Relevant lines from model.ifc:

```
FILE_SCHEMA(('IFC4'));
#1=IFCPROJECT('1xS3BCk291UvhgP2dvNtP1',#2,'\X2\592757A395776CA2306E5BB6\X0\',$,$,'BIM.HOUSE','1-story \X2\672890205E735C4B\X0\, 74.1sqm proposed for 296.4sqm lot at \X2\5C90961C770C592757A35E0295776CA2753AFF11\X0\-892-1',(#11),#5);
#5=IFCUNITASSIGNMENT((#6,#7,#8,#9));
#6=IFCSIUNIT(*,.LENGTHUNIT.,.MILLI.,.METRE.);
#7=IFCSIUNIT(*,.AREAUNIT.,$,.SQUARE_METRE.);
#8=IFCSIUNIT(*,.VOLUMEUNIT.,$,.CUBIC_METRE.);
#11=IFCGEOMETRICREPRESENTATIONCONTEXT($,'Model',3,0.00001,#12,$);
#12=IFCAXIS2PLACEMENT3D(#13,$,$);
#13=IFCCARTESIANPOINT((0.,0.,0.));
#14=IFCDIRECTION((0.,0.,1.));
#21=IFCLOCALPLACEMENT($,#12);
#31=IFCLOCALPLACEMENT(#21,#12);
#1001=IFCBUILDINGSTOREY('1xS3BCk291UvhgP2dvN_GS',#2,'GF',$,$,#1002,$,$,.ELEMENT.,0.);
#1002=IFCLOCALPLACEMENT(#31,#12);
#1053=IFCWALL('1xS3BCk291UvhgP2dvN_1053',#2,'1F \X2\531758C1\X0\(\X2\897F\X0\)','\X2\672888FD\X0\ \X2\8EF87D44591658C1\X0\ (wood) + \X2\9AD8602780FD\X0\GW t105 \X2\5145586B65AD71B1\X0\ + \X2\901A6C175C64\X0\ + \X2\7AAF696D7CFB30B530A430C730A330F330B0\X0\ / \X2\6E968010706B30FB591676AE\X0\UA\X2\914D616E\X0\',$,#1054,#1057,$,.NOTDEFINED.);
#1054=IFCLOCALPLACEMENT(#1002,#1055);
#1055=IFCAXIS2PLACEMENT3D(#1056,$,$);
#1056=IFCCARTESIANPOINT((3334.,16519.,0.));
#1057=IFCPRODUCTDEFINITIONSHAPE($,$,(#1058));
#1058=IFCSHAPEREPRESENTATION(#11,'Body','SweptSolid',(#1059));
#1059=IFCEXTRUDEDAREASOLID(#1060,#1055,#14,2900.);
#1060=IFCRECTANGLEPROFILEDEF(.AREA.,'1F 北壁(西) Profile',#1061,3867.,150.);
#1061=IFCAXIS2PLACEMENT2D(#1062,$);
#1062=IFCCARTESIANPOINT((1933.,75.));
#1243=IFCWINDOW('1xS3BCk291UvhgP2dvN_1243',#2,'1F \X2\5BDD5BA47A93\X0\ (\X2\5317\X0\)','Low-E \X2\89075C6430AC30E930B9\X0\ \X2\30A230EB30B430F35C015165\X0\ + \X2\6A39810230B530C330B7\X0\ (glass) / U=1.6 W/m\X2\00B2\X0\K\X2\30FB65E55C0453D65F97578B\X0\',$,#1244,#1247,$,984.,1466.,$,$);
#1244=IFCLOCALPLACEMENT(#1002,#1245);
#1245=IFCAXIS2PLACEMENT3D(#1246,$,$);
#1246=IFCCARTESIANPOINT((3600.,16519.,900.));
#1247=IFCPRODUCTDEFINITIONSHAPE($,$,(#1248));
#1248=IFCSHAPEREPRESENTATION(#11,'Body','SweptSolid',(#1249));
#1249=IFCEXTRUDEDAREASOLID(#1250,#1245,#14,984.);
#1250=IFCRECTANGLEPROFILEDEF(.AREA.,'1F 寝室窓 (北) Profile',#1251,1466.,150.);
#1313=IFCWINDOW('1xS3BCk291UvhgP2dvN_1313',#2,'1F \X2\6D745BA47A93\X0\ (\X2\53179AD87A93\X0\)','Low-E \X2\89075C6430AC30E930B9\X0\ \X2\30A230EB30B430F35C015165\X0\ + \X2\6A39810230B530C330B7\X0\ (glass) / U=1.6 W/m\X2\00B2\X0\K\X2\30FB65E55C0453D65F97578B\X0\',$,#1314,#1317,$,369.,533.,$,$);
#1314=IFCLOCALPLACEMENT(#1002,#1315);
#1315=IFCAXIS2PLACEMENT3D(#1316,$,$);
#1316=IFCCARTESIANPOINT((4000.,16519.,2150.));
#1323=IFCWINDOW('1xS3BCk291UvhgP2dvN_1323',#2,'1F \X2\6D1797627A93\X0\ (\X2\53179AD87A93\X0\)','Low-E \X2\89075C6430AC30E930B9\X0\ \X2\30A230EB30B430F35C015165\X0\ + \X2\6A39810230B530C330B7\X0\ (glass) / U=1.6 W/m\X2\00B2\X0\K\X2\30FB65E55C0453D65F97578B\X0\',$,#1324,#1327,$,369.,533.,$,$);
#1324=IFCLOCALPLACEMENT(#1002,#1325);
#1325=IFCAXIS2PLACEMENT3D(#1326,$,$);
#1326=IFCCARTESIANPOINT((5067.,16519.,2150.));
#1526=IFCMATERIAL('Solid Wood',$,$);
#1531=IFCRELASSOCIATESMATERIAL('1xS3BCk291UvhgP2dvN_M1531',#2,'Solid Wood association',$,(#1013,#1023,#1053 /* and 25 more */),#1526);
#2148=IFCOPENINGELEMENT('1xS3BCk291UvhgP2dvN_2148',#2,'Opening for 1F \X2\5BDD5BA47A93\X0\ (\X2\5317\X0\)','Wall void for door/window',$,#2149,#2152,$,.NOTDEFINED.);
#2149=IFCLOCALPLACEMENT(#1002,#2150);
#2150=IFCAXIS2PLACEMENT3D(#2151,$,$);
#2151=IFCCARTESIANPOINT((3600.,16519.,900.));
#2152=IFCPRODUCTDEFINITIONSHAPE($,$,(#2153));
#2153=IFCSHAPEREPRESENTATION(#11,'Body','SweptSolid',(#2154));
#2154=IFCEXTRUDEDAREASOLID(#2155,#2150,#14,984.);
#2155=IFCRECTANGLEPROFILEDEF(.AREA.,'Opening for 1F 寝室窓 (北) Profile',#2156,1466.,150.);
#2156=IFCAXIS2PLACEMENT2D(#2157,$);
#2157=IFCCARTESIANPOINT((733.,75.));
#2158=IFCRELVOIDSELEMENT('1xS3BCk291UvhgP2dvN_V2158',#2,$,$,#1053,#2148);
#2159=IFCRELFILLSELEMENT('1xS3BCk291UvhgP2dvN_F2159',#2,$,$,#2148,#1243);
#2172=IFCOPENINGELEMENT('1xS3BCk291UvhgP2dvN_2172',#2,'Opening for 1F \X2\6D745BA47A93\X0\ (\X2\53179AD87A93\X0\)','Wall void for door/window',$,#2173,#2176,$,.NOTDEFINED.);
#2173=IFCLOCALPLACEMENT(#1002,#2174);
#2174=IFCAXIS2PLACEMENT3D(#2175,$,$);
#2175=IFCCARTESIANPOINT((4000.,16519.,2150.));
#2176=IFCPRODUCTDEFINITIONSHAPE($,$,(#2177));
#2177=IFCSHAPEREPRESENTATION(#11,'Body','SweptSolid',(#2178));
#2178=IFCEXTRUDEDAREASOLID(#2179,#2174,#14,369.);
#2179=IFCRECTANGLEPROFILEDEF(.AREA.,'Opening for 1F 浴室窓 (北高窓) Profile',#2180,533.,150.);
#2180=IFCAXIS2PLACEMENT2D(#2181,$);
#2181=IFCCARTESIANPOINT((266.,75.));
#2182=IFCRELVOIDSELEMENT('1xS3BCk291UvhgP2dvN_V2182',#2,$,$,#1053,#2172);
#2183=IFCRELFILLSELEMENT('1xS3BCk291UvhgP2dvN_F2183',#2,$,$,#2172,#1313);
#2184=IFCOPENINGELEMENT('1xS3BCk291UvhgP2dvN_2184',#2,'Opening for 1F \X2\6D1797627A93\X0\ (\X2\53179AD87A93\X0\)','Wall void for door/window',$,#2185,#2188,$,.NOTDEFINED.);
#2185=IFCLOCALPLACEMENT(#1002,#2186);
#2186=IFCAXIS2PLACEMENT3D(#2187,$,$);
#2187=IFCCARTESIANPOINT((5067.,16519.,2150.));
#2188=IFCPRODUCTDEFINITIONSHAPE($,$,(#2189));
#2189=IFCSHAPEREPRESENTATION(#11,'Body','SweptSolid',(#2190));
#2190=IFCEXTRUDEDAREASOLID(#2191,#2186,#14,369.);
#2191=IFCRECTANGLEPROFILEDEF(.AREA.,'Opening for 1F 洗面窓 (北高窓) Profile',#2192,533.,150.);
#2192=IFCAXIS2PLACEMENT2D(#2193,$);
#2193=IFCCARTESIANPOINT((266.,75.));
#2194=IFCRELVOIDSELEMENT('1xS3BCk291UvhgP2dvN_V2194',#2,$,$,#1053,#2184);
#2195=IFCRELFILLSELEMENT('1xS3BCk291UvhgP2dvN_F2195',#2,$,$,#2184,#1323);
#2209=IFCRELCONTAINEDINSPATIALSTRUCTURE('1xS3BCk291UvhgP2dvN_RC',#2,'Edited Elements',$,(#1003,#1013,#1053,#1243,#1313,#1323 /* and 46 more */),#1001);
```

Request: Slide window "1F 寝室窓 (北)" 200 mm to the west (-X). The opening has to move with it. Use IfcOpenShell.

```python
import ifcopenshell
import ifcopenshell.api.geometry
import ifcopenshell.util.placement
import ifcopenshell.util.unit

model = ifcopenshell.open("model.ifc")
unit_scale = ifcopenshell.util.unit.calculate_unit_scale(model)

window = model.by_guid("1xS3BCk291UvhgP2dvN_1243")
opening = window.FillsVoids[0].RelatingOpeningElement
wall = opening.VoidsElements[0].RelatingBuildingElement

wall_matrix = ifcopenshell.util.placement.get_local_placement(wall.ObjectPlacement)
shift = wall_matrix[:3, 0] * -0.2 / unit_scale
before = ifcopenshell.util.placement.get_local_placement(window.ObjectPlacement)[:3, 3].copy()

# The window is not placed relative to its opening, so move both.
for product in (opening, window):
    matrix = ifcopenshell.util.placement.get_local_placement(product.ObjectPlacement)
    matrix[:3, 3] += shift
    ifcopenshell.api.geometry.edit_object_placement(model, product=product, matrix=matrix, is_si=False)

after = ifcopenshell.util.placement.get_local_placement(window.ObjectPlacement)[:3, 3]
print("window moved by", (after - before).round(3) + 0.0)

model.write("model_updated.ifc")
```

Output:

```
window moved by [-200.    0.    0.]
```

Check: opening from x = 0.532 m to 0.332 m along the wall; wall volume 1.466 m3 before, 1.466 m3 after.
